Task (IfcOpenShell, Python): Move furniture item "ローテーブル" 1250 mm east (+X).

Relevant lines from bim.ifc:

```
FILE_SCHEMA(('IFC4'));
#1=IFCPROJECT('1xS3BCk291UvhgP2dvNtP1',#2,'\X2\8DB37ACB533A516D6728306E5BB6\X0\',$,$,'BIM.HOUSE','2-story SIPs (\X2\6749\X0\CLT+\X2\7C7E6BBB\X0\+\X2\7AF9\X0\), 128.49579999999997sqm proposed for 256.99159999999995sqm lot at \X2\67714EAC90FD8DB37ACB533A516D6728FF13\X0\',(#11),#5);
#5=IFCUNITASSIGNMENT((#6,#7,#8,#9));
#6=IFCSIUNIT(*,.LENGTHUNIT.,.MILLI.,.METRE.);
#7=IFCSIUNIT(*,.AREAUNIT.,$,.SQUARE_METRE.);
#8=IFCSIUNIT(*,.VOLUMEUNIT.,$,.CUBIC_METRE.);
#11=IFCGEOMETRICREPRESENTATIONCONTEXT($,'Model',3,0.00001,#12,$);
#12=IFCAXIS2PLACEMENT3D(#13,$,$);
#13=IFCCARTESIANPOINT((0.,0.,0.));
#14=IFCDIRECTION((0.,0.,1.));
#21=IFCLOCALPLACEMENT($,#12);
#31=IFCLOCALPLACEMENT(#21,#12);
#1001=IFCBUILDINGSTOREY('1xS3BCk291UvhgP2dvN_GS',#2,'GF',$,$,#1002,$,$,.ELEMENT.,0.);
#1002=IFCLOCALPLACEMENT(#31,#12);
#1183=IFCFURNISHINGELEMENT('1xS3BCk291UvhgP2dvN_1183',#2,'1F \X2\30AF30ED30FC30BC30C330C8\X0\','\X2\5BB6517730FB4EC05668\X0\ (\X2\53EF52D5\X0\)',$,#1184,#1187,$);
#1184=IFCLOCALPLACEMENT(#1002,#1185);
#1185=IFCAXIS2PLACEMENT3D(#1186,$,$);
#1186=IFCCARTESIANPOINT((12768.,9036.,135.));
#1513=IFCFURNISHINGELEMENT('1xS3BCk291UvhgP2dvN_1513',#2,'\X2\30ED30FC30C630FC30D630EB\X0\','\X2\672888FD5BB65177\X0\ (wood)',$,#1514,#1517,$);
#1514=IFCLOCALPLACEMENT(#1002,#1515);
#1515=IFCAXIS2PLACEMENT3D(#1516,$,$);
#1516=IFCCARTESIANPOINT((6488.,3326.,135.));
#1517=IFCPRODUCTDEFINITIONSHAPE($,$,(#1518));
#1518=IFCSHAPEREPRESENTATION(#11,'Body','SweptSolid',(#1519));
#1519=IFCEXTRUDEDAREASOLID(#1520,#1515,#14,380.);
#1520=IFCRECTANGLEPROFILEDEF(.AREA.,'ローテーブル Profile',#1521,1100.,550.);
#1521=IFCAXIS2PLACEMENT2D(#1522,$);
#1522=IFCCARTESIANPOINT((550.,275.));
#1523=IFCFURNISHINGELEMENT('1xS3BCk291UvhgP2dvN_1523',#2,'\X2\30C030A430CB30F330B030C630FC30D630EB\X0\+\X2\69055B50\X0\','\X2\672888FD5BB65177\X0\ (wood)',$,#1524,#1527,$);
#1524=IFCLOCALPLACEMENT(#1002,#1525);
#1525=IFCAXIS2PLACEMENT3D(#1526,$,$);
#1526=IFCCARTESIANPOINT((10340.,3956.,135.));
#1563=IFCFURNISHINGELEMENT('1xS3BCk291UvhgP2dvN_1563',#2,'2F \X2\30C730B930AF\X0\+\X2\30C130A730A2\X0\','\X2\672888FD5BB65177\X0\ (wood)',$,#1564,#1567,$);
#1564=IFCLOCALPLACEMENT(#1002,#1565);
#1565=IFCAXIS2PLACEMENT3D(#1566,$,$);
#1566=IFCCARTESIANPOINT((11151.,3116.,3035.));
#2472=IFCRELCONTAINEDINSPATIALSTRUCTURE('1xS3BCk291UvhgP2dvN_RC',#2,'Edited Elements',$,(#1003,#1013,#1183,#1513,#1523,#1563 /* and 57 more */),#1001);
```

```python
import ifcopenshell
import ifcopenshell.api.geometry
import ifcopenshell.util.placement
import ifcopenshell.util.unit

model = ifcopenshell.open("bim.ifc")
unit_scale = ifcopenshell.util.unit.calculate_unit_scale(model)

item = model.by_guid("1xS3BCk291UvhgP2dvN_1513")
matrix = ifcopenshell.util.placement.get_local_placement(item.ObjectPlacement)
matrix[0, 3] += 1.25 / unit_scale
ifcopenshell.api.geometry.edit_object_placement(model, product=item, matrix=matrix, is_si=False)

print(ifcopenshell.util.placement.get_local_placement(item.ObjectPlacement).round(3) + 0.0)

model.write("bim_updated.ifc")
```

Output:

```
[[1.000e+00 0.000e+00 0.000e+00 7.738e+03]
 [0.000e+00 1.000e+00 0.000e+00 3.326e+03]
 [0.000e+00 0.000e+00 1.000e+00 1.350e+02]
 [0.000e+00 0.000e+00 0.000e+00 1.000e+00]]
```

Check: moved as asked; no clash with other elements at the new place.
